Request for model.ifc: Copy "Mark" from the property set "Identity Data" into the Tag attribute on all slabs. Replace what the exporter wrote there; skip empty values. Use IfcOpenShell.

First a look at what the model holds.

```python
import ifcopenshell
import ifcopenshell.util.element

model = ifcopenshell.open("model.ifc")
print(model.schema)
slabs = model.by_type("IfcSlab")
print(len(slabs), "slabs")
for e in slabs[:8]:
    source = ifcopenshell.util.element.get_pset(e, "Identity Data", "Mark")
    target = e.Tag
    print(e.id(), repr(source), repr(target), sep=" | ")
```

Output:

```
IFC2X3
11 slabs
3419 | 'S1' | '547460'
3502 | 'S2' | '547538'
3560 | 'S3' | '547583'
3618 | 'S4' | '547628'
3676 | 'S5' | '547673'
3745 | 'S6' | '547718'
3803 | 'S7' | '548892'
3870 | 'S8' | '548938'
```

```python
import ifcopenshell
import ifcopenshell.util.element

model = ifcopenshell.open("model.ifc")

count = 0
for e in model.by_type("IfcSlab"):
    value = ifcopenshell.util.element.get_pset(e, "Identity Data", "Mark")
    current = e.Tag
    if not value or not value.strip() or current == value:
        continue
    e.Tag = value
    count += 1

print(count, "slabs updated")

model.write("model_v2.ifc")
```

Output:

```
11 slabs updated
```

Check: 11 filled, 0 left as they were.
